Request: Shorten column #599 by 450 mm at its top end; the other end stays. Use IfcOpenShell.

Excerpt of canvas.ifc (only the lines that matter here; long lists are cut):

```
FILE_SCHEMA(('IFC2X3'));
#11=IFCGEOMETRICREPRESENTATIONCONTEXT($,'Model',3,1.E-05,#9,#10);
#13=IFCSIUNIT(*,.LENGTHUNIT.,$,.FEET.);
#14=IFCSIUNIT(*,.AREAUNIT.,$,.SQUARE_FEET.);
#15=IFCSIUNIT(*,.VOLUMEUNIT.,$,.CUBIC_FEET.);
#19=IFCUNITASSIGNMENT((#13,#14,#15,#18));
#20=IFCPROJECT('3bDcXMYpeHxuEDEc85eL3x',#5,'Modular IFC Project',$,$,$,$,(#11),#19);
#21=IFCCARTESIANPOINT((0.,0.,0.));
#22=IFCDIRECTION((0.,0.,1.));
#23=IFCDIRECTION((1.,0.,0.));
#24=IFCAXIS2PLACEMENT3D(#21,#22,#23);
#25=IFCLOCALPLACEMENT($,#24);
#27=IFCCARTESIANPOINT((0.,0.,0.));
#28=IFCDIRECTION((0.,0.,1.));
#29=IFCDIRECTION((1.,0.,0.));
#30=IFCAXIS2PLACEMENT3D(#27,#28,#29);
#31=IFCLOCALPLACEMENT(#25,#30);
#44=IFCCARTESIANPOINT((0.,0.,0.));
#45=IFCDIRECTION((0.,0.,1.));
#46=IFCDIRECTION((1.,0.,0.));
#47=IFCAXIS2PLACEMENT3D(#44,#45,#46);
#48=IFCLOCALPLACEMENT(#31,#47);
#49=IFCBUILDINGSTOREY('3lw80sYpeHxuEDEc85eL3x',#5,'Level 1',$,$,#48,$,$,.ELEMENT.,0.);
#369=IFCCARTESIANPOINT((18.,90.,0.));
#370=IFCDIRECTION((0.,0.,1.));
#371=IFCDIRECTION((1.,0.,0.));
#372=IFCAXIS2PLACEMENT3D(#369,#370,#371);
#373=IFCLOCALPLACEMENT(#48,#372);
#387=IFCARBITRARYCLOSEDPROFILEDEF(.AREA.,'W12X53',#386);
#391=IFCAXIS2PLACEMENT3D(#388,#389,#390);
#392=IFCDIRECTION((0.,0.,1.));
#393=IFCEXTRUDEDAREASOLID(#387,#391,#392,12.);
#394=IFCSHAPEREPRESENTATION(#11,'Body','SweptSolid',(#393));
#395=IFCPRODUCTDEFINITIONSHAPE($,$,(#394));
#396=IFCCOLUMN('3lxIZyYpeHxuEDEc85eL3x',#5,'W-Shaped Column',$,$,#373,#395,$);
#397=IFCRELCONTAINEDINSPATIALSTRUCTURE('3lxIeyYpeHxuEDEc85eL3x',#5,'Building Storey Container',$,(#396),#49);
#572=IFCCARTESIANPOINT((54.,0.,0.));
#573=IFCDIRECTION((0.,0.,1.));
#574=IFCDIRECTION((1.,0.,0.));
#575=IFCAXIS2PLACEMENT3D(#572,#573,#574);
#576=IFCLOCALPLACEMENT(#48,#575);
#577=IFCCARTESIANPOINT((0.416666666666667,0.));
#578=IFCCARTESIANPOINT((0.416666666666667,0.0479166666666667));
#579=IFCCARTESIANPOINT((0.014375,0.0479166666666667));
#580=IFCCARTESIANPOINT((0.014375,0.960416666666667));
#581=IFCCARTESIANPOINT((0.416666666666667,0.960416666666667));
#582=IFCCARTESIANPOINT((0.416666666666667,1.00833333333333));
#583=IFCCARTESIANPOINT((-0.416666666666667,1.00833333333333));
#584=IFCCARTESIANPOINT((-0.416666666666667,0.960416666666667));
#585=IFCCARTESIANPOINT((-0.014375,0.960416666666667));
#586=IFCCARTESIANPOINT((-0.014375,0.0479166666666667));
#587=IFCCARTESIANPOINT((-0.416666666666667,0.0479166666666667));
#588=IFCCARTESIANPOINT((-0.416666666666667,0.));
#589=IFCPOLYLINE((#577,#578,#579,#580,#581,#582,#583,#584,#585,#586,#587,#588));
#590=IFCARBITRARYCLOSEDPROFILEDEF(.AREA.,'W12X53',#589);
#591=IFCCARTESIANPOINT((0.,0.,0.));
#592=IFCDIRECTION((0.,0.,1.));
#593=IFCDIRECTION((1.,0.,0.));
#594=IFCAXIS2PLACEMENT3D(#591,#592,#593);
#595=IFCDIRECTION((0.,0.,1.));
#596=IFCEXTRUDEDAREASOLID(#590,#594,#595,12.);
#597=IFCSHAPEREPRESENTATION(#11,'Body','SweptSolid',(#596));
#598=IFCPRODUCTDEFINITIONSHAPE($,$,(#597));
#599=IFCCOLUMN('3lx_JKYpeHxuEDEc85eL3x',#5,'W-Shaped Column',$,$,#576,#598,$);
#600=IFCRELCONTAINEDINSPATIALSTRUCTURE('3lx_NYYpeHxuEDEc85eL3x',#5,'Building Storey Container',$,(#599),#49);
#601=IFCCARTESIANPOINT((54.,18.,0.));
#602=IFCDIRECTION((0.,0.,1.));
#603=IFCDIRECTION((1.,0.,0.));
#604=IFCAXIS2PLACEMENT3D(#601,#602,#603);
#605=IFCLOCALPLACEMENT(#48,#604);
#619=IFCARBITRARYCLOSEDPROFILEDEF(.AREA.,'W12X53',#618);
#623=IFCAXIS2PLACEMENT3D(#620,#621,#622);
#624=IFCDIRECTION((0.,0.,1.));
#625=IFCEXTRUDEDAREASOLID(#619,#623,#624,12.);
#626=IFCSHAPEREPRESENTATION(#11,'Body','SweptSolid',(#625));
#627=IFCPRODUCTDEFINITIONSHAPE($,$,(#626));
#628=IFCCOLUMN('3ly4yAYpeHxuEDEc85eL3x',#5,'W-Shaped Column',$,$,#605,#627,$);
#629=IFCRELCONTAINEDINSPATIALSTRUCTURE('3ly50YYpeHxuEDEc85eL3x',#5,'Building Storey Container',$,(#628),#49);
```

```python
import ifcopenshell
import ifcopenshell.util.unit

model = ifcopenshell.open("canvas.ifc")
unit_scale = ifcopenshell.util.unit.calculate_unit_scale(model)

member = model.by_guid("3lx_JKYpeHxuEDEc85eL3x")
change = -0.45 / unit_scale

# The extrusion runs towards the end named, so only its depth changes.
body = next(r for r in member.Representation.Representations if r.RepresentationIdentifier == "Body")
solid = body.Items[0]
old_length = solid.Depth
solid.Depth += change

print(f"length {old_length:g} -> {solid.Depth:g}")

model.write("canvas_v2.ifc")
```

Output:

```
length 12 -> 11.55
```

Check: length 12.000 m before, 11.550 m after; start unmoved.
